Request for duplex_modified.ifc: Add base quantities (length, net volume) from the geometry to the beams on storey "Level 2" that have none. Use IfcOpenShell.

First a look at what the model holds.

```python
import ifcopenshell
import ifcopenshell.util.element
import ifcopenshell.util.unit

model = ifcopenshell.open("duplex_modified.ifc")
print(model.schema)
for unit_type in ("LENGTHUNIT", "AREAUNIT", "VOLUMEUNIT"):
    print(unit_type, ifcopenshell.util.unit.calculate_unit_scale(model, unit_type))
storey = next(s for s in model.by_type("IfcBuildingStorey") if s.Name == "Level 2")
beams = [e for e in ifcopenshell.util.element.get_decomposition(storey) if e.is_a("IfcBeam")]
for e in sorted(beams, key=lambda e: e.id()):
    print(e.id(), e.is_a(), e.Name, list(ifcopenshell.util.element.get_psets(e, qtos_only=True)), sep=" | ")
```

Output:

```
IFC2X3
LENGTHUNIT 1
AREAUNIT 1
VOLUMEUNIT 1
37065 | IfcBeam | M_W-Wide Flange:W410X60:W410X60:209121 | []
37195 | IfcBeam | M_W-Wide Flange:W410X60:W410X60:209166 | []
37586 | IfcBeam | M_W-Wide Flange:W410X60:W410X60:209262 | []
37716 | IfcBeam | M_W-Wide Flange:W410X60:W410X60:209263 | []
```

```python
import ifcopenshell
import ifcopenshell.api.pset
import ifcopenshell.geom
import ifcopenshell.util.element
import ifcopenshell.util.shape
import ifcopenshell.util.unit

model = ifcopenshell.open("duplex_modified.ifc")
unit_scale = ifcopenshell.util.unit.calculate_unit_scale(model)
volume_scale = ifcopenshell.util.unit.calculate_unit_scale(model, "VOLUMEUNIT")
settings = ifcopenshell.geom.settings()

storey = next(s for s in model.by_type("IfcBuildingStorey") if s.Name == "Level 2")
beams = [e for e in ifcopenshell.util.element.get_decomposition(storey) if e.is_a("IfcBeam")]

for e in sorted(beams, key=lambda e: e.id()):
    if ifcopenshell.util.element.get_psets(e, qtos_only=True, should_inherit=False):
        continue
    # Geometry comes back in metres, in the element's own axes.
    shape = ifcopenshell.geom.create_shape(settings, e)
    values = {
        "Length": ifcopenshell.util.shape.get_max_xyz(shape.geometry) / unit_scale,
        "NetVolume": ifcopenshell.util.shape.get_volume(shape.geometry) / volume_scale,
    }
    qto = ifcopenshell.api.pset.add_qto(model, product=e, name="BaseQuantities")
    ifcopenshell.api.pset.edit_qto(model, qto=qto, properties=values)
    print(e.id(), {k: round(v, 3) for k, v in values.items()})

model.write("duplex_modified-out.ifc")
```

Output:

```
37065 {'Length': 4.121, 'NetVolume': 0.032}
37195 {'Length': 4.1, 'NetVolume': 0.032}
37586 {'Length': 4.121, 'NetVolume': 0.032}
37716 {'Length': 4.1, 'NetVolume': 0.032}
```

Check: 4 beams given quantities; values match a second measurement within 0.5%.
